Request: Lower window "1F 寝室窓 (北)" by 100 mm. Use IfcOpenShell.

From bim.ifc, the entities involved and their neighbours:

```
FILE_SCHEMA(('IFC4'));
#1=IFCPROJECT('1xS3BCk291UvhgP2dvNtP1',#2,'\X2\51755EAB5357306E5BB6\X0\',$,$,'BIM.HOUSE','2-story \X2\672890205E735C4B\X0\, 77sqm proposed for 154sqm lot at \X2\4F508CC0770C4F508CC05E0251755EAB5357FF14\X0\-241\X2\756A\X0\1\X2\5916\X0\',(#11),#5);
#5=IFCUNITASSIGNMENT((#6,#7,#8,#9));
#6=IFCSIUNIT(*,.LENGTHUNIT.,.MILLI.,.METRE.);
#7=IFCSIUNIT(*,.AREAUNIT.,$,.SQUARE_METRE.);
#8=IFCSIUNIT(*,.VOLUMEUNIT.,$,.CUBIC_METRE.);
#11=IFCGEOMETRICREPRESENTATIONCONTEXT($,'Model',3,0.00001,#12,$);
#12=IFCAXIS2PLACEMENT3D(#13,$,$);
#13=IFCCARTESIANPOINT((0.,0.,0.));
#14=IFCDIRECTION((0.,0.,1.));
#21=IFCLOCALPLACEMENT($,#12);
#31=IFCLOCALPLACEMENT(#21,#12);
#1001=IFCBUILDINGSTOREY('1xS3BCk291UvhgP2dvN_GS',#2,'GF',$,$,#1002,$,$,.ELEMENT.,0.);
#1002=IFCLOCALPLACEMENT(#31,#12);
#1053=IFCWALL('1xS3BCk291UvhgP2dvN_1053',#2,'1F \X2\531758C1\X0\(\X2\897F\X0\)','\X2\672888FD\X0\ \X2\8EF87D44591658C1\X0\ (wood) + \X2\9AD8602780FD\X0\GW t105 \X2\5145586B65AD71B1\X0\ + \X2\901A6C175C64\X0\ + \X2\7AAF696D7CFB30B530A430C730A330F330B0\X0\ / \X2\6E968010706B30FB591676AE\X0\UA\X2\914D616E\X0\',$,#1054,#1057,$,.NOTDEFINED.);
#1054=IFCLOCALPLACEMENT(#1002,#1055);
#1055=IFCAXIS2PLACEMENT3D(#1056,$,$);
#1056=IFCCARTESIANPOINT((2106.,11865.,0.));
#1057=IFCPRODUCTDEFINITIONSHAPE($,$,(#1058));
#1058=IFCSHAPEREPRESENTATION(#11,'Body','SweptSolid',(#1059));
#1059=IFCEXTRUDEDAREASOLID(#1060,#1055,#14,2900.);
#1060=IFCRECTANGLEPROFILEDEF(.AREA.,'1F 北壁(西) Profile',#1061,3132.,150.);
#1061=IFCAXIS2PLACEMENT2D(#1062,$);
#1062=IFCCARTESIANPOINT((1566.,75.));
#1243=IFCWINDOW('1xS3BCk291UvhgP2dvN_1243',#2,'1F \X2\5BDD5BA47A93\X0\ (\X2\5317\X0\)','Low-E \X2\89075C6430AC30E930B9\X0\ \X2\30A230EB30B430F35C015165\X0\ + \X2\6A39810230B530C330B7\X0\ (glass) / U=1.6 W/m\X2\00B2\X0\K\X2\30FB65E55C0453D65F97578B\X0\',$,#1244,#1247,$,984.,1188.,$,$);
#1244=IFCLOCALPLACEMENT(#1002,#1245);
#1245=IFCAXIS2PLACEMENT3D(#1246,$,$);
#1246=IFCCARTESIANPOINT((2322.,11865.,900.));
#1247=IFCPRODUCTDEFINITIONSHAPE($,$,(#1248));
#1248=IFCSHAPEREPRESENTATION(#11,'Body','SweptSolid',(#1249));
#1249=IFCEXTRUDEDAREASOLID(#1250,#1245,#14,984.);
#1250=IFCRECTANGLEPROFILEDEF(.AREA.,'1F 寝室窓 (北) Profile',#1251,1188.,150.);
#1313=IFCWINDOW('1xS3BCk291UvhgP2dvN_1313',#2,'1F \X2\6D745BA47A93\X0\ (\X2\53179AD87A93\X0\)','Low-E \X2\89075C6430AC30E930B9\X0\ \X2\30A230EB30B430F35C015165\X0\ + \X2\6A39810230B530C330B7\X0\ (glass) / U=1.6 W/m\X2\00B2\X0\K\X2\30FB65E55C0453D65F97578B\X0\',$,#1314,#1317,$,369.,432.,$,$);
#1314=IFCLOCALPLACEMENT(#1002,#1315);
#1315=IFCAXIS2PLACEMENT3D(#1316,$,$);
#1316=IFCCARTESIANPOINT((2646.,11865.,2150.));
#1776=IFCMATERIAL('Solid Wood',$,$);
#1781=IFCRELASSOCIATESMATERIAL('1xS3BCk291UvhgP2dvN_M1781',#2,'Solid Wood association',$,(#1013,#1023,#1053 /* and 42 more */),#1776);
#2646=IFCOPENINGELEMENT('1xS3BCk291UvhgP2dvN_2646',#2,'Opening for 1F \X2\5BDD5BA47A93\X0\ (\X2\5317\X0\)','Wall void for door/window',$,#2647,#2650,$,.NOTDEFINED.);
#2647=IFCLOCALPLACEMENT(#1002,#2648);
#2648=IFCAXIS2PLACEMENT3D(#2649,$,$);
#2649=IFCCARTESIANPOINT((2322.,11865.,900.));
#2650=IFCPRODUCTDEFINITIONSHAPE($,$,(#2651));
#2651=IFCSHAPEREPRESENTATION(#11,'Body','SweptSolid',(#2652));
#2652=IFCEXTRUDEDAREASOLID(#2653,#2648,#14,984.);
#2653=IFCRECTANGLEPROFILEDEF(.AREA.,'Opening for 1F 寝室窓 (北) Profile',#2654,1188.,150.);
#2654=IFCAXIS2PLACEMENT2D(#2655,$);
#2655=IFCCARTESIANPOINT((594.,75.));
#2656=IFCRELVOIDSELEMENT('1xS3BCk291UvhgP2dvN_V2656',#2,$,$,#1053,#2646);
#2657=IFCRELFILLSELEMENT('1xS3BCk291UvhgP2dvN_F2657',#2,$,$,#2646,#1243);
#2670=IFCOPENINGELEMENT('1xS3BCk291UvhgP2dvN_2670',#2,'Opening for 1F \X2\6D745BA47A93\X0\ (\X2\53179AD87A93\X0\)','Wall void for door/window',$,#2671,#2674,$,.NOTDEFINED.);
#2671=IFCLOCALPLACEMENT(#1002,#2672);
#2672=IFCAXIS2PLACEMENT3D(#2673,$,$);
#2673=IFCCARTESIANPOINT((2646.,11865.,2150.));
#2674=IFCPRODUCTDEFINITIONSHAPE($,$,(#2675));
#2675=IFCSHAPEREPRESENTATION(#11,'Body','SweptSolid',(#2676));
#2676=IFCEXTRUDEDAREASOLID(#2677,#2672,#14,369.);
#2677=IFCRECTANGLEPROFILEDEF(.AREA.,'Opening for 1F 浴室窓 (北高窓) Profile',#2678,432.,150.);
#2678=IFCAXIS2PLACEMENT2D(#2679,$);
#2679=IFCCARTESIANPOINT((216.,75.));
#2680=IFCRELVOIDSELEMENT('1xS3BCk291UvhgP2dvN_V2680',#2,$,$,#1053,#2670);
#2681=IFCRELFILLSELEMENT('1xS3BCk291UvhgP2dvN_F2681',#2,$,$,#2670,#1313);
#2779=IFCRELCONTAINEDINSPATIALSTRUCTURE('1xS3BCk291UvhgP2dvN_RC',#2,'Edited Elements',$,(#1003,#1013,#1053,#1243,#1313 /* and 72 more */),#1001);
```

```python
import numpy as np
import ifcopenshell
import ifcopenshell.api.geometry
import ifcopenshell.util.placement
import ifcopenshell.util.unit

model = ifcopenshell.open("bim.ifc")
unit_scale = ifcopenshell.util.unit.calculate_unit_scale(model)

window = model.by_guid("1xS3BCk291UvhgP2dvN_1243")
opening = window.FillsVoids[0].RelatingOpeningElement
dz = -0.1 / unit_scale

shift = np.array([0.0, 0.0, dz])
# The window is not placed relative to its opening, so move both.
for product in (opening, window):
    matrix = ifcopenshell.util.placement.get_local_placement(product.ObjectPlacement)
    matrix[:3, 3] += shift
    ifcopenshell.api.geometry.edit_object_placement(model, product=product, matrix=matrix, is_si=False)

print(f"moved by {dz * unit_scale:+.3f} m")

model.write("bim_edited.ifc")
```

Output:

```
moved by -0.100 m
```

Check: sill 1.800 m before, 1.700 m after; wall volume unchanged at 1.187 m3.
